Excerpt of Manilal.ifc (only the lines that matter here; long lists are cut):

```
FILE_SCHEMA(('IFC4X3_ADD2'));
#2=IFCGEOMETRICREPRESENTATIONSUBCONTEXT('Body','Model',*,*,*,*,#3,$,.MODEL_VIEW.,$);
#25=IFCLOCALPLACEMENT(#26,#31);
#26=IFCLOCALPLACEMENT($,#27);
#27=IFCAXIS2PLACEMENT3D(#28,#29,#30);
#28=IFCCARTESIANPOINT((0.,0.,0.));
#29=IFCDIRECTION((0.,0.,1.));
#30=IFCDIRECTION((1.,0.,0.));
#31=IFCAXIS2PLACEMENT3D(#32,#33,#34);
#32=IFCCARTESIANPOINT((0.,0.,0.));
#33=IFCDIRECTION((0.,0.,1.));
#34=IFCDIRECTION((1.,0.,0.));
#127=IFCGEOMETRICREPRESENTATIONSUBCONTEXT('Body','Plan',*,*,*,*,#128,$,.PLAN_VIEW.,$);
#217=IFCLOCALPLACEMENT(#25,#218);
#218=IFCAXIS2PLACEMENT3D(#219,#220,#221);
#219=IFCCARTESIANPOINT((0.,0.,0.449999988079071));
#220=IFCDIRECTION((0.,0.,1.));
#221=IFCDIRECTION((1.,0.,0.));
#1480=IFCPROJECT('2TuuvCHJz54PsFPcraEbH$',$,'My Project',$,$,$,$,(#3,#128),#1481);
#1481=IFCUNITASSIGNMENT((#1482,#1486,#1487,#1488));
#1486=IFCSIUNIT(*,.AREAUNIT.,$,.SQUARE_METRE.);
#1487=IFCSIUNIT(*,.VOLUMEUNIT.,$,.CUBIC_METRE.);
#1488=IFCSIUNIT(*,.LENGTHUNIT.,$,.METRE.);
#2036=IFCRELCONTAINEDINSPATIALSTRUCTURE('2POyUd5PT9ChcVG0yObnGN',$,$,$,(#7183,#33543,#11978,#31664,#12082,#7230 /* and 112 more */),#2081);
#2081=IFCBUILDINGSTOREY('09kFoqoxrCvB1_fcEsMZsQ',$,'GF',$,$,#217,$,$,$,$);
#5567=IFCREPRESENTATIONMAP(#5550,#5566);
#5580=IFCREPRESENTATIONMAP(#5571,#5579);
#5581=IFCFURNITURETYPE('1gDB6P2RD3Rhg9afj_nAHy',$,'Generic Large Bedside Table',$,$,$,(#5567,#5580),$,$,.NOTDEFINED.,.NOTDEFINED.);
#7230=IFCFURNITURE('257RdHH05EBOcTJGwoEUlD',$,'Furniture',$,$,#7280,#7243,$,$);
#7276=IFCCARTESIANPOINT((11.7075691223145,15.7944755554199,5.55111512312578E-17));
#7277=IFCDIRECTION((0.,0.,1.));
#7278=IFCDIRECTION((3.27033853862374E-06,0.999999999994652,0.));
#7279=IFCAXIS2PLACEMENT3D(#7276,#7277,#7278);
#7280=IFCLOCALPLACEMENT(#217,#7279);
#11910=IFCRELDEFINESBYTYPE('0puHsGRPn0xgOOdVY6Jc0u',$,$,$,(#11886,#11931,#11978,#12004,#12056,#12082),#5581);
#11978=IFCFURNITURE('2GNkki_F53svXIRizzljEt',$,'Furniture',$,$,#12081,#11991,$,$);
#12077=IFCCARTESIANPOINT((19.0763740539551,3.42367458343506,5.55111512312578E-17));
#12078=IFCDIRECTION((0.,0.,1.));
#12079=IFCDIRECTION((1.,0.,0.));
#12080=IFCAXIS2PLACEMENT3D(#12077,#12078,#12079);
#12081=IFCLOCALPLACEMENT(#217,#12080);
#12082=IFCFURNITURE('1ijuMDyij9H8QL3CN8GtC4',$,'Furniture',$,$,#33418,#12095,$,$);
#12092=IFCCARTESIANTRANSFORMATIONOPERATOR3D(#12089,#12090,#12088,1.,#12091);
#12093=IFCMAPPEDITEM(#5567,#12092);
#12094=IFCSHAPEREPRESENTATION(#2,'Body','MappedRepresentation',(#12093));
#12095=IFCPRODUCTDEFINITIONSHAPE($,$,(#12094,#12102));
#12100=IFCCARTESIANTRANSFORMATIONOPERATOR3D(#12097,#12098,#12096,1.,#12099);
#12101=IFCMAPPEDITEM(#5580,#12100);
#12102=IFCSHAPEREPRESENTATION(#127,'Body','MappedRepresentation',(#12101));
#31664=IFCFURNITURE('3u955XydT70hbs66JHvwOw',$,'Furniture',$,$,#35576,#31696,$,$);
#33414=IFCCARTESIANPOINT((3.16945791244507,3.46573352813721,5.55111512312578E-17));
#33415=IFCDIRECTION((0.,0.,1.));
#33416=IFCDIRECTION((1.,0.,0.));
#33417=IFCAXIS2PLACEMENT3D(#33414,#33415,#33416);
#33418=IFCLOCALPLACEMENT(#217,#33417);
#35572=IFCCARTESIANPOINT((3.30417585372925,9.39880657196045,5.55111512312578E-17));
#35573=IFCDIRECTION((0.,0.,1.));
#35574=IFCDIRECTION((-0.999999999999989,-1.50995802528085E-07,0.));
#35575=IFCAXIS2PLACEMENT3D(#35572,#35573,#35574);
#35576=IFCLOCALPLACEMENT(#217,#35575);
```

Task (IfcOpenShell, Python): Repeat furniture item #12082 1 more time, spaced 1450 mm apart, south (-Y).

```python
import numpy as np
import ifcopenshell
import ifcopenshell.api.geometry
import ifcopenshell.api.root
import ifcopenshell.util.element
import ifcopenshell.util.placement
import ifcopenshell.util.unit

model = ifcopenshell.open("Manilal.ifc")
unit_scale = ifcopenshell.util.unit.calculate_unit_scale(model)

source = model.by_guid("1ijuMDyij9H8QL3CN8GtC4")
base = ifcopenshell.util.placement.get_local_placement(source.ObjectPlacement)
step = np.array([0.0, -1.0, 0.0]) * 1.45 / unit_scale

for i in range(1, 2):
    copy = ifcopenshell.api.root.copy_class(model, product=source)
    copy.Representation = ifcopenshell.util.element.copy_deep(
        model, source.Representation, exclude=["IfcGeometricRepresentationContext", "IfcRepresentationMap"]
    )
    matrix = base.copy()
    matrix[:3, 3] += i * step
    print("added at", matrix[:3, 3].round(3) + 0.0)
    ifcopenshell.api.geometry.edit_object_placement(model, product=copy, matrix=matrix, is_si=False)

model.write("Manilal_updated.ifc")
```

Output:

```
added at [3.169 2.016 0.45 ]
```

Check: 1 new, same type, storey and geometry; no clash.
